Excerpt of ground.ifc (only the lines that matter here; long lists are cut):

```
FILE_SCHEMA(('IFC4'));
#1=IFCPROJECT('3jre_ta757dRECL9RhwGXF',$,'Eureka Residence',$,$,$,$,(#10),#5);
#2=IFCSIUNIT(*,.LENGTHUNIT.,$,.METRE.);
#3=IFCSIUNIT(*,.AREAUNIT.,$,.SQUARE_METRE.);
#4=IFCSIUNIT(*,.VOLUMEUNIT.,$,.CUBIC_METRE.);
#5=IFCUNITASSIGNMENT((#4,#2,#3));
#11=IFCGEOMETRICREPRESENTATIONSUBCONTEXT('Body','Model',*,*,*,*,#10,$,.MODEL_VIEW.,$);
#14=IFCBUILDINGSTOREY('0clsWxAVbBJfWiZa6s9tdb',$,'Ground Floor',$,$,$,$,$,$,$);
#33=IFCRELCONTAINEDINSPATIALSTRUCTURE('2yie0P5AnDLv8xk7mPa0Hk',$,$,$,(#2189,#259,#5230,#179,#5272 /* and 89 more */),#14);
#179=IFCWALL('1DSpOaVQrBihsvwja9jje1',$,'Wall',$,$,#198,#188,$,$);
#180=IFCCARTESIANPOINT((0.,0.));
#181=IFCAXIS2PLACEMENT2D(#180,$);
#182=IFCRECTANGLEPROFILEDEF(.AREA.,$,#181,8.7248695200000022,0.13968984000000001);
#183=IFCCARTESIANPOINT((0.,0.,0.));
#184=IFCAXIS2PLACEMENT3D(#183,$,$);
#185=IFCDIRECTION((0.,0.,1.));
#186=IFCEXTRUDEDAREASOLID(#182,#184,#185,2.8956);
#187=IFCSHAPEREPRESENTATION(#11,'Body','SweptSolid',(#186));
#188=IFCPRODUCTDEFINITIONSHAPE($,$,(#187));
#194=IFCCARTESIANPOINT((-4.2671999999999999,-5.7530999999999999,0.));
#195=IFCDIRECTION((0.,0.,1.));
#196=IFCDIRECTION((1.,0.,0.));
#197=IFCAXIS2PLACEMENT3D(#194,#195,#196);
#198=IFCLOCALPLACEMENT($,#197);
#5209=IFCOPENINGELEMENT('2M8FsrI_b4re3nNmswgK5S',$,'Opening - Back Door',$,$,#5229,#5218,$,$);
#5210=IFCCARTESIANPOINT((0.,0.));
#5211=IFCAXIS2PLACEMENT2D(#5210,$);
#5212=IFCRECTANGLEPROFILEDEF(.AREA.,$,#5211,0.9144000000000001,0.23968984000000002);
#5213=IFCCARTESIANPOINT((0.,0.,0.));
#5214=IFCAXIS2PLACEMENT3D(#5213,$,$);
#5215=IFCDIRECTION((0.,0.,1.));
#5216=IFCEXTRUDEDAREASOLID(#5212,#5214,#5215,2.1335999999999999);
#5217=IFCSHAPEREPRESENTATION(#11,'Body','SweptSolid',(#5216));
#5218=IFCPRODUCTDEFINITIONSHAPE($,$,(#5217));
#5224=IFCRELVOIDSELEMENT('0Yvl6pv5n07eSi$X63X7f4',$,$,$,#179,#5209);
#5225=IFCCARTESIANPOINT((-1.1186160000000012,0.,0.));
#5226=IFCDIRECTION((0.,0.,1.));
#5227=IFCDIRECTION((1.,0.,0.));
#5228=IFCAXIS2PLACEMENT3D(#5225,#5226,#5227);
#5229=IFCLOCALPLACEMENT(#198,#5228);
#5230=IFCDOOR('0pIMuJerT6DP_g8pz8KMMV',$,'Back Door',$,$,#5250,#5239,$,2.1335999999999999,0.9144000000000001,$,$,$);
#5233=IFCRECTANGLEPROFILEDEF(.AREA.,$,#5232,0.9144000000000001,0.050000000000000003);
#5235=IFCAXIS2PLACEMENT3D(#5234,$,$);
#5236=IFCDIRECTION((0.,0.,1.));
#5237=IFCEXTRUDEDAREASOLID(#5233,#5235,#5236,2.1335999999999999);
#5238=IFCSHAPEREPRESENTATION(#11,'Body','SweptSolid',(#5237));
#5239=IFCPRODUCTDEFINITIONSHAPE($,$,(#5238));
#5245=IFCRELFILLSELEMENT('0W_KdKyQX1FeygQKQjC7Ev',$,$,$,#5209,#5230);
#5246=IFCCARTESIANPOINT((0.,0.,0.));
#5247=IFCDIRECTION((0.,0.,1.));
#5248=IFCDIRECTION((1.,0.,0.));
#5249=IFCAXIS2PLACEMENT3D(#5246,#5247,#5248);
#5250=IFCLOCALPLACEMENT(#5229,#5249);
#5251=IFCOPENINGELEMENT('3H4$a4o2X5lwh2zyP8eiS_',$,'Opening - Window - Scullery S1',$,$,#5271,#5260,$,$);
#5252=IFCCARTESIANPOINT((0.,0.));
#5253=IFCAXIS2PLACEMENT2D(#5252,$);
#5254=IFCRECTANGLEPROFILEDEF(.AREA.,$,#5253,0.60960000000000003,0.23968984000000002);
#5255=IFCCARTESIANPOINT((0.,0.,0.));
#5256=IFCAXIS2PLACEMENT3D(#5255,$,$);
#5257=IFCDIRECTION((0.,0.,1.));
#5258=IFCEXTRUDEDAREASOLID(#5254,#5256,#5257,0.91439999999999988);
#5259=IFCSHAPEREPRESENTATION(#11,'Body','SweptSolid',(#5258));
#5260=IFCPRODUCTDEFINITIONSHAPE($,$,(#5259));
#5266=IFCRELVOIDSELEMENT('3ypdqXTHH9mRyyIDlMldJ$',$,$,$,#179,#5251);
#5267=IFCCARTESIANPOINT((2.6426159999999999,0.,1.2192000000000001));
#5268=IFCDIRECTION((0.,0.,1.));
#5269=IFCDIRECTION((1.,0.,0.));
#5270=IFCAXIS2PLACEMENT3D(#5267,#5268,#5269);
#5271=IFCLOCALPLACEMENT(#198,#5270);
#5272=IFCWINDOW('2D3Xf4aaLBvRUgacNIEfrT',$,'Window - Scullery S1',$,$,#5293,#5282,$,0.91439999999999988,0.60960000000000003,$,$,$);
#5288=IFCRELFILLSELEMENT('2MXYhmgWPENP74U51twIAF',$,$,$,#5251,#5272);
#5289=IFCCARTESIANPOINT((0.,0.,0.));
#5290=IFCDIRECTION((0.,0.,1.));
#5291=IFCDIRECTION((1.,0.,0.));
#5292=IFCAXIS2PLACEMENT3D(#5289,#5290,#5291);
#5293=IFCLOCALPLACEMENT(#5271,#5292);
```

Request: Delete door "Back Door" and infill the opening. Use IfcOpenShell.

```python
import ifcopenshell
import ifcopenshell.api.feature
import ifcopenshell.api.root
import ifcopenshell.geom
import ifcopenshell.util.shape

model = ifcopenshell.open("ground.ifc")
settings = ifcopenshell.geom.settings()


def volume(element):
    """Net volume in cubic metres, openings subtracted."""
    shape = ifcopenshell.geom.create_shape(settings, element)
    return ifcopenshell.util.shape.get_volume(shape.geometry)


door = model.by_guid("0pIMuJerT6DP_g8pz8KMMV")
opening = door.FillsVoids[0].RelatingOpeningElement
wall = opening.VoidsElements[0].RelatingBuildingElement
before = volume(wall)

ifcopenshell.api.root.remove_product(model, product=door)
ifcopenshell.api.feature.remove_feature(model, feature=opening)

after = volume(wall)

print(f"wall volume {before:.3f} -> {after:.3f} m3")

model.write("ground-out.ifc")
```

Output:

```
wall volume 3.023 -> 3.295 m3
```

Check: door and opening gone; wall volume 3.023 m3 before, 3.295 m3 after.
